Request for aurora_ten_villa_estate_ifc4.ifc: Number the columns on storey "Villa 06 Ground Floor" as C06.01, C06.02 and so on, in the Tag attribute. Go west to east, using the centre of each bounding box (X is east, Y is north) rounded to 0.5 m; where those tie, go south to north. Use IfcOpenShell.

First a look at what the model holds.

```python
import ifcopenshell
import ifcopenshell.util.element
import ifcopenshell.util.placement

model = ifcopenshell.open("aurora_ten_villa_estate_ifc4.ifc")
print(model.schema)
storey = next(s for s in model.by_type("IfcBuildingStorey") if s.Name == "Villa 06 Ground Floor")
columns = [e for e in ifcopenshell.util.element.get_decomposition(storey) if e.is_a("IfcColumn")]
for e in sorted(columns, key=lambda e: e.id()):
    origin = ifcopenshell.util.placement.get_local_placement(e.ObjectPlacement)[:3, 3]
    print(e.id(), e.Tag, e.Name, origin.round(2) + 0.0, sep=" | ")
```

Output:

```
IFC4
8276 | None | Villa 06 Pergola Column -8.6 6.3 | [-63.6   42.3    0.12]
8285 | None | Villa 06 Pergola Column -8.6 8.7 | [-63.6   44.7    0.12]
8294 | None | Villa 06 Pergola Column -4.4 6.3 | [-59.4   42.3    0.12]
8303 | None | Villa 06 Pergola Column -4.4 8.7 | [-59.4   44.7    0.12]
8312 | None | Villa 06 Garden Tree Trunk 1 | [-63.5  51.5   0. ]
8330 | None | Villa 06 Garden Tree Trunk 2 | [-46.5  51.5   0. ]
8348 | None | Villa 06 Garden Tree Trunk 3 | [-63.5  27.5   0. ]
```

```python
import ifcopenshell
import ifcopenshell.geom
import ifcopenshell.util.element
import ifcopenshell.util.shape

model = ifcopenshell.open("aurora_ten_villa_estate_ifc4.ifc")
settings = ifcopenshell.geom.settings()
settings.set("use-world-coords", True)


def centre(element):
    shape = ifcopenshell.geom.create_shape(settings, element)
    return ifcopenshell.util.shape.get_bbox_centroid(shape.geometry)


storey = next(s for s in model.by_type("IfcBuildingStorey") if s.Name == "Villa 06 Ground Floor")
columns = [e for e in ifcopenshell.util.element.get_decomposition(storey) if e.is_a("IfcColumn")]

# Insertion points can sit at a corner or the storey origin, so sort by the geometry (in metres).
centres = {e: centre(e) for e in columns}
columns.sort(key=lambda e: (round(centres[e][0] / 0.5), centres[e][1]))

for i, e in enumerate(columns, start=1):
    number = f"C06.{i:02d}"
    e.Tag = number
    print(e.id(), number)

model.write("aurora_ten_villa_estate_ifc4_v2.ifc")
```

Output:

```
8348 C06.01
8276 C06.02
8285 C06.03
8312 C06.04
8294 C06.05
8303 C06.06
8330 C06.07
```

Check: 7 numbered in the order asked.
